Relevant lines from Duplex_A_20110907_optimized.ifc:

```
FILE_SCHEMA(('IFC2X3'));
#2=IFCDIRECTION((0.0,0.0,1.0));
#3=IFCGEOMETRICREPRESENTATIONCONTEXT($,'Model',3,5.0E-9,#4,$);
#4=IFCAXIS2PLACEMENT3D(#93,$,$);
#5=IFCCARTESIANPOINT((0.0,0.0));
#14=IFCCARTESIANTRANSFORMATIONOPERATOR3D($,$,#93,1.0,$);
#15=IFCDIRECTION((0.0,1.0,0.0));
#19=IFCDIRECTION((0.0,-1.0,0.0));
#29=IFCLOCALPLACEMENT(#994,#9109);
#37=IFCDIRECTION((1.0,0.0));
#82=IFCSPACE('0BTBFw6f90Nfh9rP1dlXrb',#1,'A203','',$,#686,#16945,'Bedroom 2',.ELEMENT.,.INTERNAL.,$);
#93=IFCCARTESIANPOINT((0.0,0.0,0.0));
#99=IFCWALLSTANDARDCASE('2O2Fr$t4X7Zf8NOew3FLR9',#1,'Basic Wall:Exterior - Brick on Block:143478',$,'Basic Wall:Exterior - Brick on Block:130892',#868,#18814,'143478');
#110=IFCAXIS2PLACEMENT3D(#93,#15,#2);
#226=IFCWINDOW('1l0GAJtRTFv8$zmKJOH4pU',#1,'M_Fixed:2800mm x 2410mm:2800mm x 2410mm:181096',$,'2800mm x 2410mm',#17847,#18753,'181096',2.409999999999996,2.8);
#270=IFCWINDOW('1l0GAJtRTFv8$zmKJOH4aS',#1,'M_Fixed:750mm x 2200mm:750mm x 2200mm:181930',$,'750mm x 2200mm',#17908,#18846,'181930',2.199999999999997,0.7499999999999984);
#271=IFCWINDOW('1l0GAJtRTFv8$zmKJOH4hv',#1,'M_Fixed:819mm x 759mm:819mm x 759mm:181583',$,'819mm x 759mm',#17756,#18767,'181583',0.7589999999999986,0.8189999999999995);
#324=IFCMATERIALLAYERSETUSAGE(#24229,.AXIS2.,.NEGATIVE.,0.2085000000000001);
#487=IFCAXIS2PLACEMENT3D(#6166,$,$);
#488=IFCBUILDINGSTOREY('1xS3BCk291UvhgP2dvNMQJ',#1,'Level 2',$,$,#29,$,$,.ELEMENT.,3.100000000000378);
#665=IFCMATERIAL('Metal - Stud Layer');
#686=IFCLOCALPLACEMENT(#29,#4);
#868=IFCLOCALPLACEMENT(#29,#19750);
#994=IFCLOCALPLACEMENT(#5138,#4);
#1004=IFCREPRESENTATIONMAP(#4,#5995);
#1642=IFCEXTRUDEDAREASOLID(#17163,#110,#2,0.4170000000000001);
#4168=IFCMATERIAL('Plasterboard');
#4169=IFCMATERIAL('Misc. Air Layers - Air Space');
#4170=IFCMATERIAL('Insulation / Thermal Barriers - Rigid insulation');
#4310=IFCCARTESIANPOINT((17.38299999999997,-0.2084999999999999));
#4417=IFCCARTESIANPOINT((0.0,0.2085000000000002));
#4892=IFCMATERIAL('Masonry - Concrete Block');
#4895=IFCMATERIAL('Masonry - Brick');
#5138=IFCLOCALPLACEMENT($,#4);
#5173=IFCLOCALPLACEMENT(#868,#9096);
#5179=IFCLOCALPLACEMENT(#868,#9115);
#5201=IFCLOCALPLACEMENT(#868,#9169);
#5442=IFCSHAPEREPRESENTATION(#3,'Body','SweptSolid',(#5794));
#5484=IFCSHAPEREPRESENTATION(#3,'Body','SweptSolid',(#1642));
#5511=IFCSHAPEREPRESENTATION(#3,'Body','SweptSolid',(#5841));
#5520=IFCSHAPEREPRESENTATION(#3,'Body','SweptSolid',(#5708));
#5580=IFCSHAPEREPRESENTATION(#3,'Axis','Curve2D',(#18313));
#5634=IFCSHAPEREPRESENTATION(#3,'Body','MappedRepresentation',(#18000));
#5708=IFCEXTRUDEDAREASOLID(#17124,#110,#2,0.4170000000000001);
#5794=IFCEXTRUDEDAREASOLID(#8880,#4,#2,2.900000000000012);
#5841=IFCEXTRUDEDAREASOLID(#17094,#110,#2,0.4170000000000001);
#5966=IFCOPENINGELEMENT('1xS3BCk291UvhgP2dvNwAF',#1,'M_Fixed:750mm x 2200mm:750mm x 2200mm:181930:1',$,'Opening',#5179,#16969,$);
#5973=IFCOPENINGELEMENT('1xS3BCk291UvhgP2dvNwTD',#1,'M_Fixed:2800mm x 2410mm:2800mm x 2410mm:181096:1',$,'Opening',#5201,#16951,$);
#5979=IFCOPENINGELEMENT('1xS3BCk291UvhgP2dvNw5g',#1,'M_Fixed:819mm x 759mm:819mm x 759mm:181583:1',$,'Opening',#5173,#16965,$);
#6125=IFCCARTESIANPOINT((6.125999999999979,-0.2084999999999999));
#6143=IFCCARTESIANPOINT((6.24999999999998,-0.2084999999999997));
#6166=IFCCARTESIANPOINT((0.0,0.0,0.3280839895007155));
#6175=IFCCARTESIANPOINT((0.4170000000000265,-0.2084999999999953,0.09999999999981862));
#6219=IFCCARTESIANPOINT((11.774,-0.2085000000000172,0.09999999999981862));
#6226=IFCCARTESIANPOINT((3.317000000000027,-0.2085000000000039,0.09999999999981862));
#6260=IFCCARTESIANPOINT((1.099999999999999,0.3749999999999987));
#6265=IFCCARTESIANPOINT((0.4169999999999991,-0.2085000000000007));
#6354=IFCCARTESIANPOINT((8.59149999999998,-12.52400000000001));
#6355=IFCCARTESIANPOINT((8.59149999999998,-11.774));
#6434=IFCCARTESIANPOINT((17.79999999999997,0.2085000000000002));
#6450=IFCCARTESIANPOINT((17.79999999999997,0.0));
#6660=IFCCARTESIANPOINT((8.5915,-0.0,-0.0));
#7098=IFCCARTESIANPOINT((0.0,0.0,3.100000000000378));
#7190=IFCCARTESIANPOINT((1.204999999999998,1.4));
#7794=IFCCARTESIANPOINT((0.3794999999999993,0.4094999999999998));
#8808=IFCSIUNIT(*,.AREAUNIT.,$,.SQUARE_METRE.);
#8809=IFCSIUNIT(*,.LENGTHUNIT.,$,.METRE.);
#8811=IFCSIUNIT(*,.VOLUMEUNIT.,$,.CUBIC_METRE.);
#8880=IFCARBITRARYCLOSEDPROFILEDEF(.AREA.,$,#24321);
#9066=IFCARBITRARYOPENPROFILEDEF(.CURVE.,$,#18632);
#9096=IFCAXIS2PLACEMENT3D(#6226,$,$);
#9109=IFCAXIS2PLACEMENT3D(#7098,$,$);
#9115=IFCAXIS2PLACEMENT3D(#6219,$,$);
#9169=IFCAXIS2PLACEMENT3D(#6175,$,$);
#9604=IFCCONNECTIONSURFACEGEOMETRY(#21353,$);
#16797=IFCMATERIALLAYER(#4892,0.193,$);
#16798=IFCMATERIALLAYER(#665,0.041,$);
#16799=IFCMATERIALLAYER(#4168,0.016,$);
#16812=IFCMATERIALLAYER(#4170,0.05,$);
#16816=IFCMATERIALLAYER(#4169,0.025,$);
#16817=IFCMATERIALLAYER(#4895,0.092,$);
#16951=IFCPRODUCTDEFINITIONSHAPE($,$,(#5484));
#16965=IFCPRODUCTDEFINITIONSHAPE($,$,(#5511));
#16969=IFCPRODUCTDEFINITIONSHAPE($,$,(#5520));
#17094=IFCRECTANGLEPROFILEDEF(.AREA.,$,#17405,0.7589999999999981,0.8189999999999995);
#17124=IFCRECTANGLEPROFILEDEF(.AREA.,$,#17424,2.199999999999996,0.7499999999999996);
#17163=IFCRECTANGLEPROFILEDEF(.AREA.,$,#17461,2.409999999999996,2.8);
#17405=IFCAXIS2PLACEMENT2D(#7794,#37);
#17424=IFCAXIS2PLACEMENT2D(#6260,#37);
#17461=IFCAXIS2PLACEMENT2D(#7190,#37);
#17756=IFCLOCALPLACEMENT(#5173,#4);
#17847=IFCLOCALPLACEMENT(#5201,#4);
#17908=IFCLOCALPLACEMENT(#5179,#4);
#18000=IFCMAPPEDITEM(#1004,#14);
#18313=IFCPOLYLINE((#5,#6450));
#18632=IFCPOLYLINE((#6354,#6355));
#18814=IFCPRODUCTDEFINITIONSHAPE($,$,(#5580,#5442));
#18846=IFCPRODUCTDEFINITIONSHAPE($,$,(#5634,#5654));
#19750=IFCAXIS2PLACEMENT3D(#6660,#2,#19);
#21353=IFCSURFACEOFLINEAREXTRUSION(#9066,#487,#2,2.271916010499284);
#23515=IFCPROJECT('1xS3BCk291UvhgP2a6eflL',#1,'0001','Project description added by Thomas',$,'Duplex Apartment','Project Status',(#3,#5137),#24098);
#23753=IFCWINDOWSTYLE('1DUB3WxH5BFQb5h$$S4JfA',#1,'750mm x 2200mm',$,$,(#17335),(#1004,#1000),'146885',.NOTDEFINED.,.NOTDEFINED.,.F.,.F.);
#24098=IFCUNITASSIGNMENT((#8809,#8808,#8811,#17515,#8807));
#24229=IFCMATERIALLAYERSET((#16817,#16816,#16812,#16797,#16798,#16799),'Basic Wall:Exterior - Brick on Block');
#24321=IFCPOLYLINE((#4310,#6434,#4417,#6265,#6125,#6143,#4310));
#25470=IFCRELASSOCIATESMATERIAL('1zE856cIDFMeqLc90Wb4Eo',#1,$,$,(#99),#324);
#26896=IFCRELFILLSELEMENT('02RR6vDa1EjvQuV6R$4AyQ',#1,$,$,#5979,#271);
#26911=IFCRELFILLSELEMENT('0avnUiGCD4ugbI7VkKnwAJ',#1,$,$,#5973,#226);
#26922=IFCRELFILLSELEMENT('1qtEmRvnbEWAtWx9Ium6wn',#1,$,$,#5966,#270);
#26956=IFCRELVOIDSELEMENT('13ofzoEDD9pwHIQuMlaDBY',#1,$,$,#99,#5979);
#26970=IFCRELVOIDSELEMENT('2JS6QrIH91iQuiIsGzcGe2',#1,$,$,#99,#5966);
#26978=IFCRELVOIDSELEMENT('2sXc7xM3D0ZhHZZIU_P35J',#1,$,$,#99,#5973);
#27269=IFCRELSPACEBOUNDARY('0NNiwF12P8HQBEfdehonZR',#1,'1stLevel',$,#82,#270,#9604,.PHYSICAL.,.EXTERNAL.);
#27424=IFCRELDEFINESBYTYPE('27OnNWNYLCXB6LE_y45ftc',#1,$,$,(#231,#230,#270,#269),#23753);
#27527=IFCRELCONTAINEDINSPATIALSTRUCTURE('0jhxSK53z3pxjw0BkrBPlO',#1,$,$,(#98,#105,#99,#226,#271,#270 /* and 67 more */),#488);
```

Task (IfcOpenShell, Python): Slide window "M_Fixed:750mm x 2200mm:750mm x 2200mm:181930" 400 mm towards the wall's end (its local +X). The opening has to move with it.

```python
import numpy as np
import ifcopenshell
import ifcopenshell.api.geometry
import ifcopenshell.util.placement
import ifcopenshell.util.unit

model = ifcopenshell.open("Duplex_A_20110907_optimized.ifc")
unit_scale = ifcopenshell.util.unit.calculate_unit_scale(model)

window = model.by_guid("1l0GAJtRTFv8$zmKJOH4aS")
opening = window.FillsVoids[0].RelatingOpeningElement
wall = opening.VoidsElements[0].RelatingBuildingElement

wall_matrix = ifcopenshell.util.placement.get_local_placement(wall.ObjectPlacement)
shift = wall_matrix[:3, 0] * 0.4 / unit_scale
before = ifcopenshell.util.placement.get_local_placement(window.ObjectPlacement)[:3, 3].copy()

# The window is placed relative to its opening, so it follows when the opening moves.
matrix = ifcopenshell.util.placement.get_local_placement(opening.ObjectPlacement)
matrix[:3, 3] += shift
ifcopenshell.api.geometry.edit_object_placement(
    model, product=opening, matrix=matrix, is_si=False, should_transform_children=True
)

# Space boundary surfaces are stored in each space's coordinates; move them too.
for rel in window.ProvidesBoundaries:
    if not rel.ConnectionGeometry:
        continue
    surface = rel.ConnectionGeometry.SurfaceOnRelatingElement
    space_matrix = ifcopenshell.util.placement.get_local_placement(rel.RelatingSpace.ObjectPlacement)
    point = np.array(surface.Position.Location.Coordinates) + space_matrix[:3, :3].T @ shift
    surface.Position = model.createIfcAxis2Placement3D(
        model.createIfcCartesianPoint(point.tolist()), surface.Position.Axis, surface.Position.RefDirection
    )

after = ifcopenshell.util.placement.get_local_placement(window.ObjectPlacement)[:3, 3]
print("window moved by", (after - before).round(3) + 0.0)

model.write("Duplex_A_20110907_optimized_updated.ifc")
```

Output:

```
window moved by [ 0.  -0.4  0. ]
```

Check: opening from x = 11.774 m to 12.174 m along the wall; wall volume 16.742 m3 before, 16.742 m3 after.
